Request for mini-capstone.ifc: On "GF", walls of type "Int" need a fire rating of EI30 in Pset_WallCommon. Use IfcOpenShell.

First a look at what the model holds.

```python
import ifcopenshell
import ifcopenshell.util.element

model = ifcopenshell.open("mini-capstone.ifc")
print(model.schema)
storey = next(s for s in model.by_type("IfcBuildingStorey") if s.Name == "GF")
walls = [e for e in ifcopenshell.util.element.get_decomposition(storey) if e.is_a("IfcWall")]
seen = {}
for e in walls:
    element_type = ifcopenshell.util.element.get_type(e)
    key = (element_type.Name if element_type != e and element_type else None, ifcopenshell.util.element.get_pset(e, "Pset_WallCommon", "FireRating"))
    seen[key] = seen.get(key, 0) + 1
for (name, value), count in sorted(seen.items(), key=str):
    print(count, "x", name, "|", value)
```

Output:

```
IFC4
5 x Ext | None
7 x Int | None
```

```python
import ifcopenshell
import ifcopenshell.api.pset
import ifcopenshell.util.element

model = ifcopenshell.open("mini-capstone.ifc")

storey = next(s for s in model.by_type("IfcBuildingStorey") if s.Name == "GF")
walls = [e for e in ifcopenshell.util.element.get_decomposition(storey) if e.is_a("IfcWall")]

count = 0
for e in walls:
    element_type = ifcopenshell.util.element.get_type(e)
    if element_type in (None, e) or element_type.Name != "Int":
        continue
    # add_pset returns the element's existing set when there is one.
    pset = ifcopenshell.api.pset.add_pset(model, product=e, name="Pset_WallCommon")
    ifcopenshell.api.pset.edit_pset(model, pset=pset, properties={"FireRating": "EI30"})
    count += 1

print(count, "walls updated")

model.write("mini-capstone_rev.ifc")
```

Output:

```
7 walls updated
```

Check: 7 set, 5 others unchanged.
